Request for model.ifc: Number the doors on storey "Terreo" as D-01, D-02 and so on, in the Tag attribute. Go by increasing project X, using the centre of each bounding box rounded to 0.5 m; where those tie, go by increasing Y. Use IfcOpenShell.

First a look at what the model holds.

```python
import ifcopenshell
import ifcopenshell.util.element
import ifcopenshell.util.placement

model = ifcopenshell.open("model.ifc")
print(model.schema)
storey = next(s for s in model.by_type("IfcBuildingStorey") if s.Name == "Terreo")
doors = [e for e in ifcopenshell.util.element.get_decomposition(storey) if e.is_a("IfcDoor")]
for e in sorted(doors, key=lambda e: e.id()):
    origin = ifcopenshell.util.placement.get_local_placement(e.ObjectPlacement)[:3, 3]
    print(e.id(), e.Tag, e.Name, origin.round(2) + 0.0, sep=" | ")
```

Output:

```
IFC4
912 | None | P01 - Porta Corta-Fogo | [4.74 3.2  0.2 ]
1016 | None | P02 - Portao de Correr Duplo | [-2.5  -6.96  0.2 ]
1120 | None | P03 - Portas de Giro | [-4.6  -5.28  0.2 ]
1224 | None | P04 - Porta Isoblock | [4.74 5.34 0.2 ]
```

```python
import ifcopenshell
import ifcopenshell.geom
import ifcopenshell.util.element
import ifcopenshell.util.shape

model = ifcopenshell.open("model.ifc")
settings = ifcopenshell.geom.settings()
settings.set("use-world-coords", True)


def centre(element):
    shape = ifcopenshell.geom.create_shape(settings, element)
    return ifcopenshell.util.shape.get_bbox_centroid(shape.geometry)


storey = next(s for s in model.by_type("IfcBuildingStorey") if s.Name == "Terreo")
doors = [e for e in ifcopenshell.util.element.get_decomposition(storey) if e.is_a("IfcDoor")]

# Insertion points can sit at a corner or the storey origin, so sort by the geometry (in metres).
centres = {e: centre(e) for e in doors}
doors.sort(key=lambda e: (round(centres[e][0] / 0.5), centres[e][1]))

for i, e in enumerate(doors, start=1):
    number = f"D-{i:02d}"
    e.Tag = number
    print(e.id(), number)

model.write("model_updated.ifc")
```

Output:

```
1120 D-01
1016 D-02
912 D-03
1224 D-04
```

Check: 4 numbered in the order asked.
